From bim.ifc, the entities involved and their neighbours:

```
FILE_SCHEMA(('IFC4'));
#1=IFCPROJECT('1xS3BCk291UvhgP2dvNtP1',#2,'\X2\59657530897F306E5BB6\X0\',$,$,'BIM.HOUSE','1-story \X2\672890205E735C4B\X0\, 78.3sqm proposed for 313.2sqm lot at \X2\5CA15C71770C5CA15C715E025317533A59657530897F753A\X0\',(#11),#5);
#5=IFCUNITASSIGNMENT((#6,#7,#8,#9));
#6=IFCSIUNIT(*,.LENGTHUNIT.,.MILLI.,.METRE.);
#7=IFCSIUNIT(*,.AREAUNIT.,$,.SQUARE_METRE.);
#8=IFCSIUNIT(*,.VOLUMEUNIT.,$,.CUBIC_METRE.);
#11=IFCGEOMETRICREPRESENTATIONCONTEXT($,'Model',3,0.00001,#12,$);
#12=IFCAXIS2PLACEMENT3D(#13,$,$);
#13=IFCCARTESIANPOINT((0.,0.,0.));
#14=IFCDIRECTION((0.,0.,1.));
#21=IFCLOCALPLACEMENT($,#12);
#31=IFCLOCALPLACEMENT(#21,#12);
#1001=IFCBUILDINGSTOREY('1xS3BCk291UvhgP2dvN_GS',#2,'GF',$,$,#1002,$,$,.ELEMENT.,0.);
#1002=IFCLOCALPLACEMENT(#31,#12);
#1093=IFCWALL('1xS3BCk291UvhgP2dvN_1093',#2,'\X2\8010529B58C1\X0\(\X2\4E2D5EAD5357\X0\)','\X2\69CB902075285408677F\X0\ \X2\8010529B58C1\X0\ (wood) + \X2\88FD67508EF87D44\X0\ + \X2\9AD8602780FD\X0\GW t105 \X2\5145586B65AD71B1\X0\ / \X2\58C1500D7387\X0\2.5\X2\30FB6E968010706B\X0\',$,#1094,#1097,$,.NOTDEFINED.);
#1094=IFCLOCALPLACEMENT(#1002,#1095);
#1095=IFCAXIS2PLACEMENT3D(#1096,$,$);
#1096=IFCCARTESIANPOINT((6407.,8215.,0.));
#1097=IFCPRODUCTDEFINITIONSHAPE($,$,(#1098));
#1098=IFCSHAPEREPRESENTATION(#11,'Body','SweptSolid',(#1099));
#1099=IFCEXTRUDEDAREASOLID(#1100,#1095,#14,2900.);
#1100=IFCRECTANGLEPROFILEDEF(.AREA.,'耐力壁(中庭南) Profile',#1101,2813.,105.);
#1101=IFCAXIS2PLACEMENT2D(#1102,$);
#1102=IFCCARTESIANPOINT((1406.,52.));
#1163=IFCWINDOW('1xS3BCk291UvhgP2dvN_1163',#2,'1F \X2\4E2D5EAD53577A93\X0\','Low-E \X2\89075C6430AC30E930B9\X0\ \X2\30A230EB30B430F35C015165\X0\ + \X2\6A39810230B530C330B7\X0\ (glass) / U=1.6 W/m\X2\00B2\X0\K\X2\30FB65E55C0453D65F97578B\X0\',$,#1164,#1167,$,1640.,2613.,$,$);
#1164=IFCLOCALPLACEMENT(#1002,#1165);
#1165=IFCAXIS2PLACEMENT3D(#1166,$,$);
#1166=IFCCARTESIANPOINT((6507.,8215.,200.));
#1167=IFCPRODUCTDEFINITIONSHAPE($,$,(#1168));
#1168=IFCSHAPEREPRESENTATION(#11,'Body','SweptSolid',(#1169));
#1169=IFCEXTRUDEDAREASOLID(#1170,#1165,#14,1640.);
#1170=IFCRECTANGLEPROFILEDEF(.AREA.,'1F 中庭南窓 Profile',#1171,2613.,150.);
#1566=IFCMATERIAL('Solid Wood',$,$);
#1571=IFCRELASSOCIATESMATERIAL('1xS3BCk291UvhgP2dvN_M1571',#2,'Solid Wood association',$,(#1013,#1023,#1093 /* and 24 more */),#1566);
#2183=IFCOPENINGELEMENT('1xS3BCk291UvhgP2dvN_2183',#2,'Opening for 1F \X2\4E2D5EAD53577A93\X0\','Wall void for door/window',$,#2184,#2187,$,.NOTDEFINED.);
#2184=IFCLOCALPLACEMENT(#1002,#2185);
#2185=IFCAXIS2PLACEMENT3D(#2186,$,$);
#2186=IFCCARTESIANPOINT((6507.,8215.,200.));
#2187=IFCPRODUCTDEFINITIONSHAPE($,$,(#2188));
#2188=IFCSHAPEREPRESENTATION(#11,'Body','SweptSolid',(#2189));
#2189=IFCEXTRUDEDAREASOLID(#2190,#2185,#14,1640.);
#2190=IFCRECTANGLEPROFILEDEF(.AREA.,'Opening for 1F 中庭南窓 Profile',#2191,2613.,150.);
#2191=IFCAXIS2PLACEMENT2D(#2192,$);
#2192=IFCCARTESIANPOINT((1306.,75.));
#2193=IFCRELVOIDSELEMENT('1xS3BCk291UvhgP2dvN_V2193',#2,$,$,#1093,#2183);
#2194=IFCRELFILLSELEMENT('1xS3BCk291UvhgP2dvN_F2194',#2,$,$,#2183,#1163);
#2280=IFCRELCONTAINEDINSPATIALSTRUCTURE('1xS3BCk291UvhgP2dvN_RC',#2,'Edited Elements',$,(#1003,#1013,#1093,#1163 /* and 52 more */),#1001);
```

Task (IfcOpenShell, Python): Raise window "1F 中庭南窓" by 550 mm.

```python
import numpy as np
import ifcopenshell
import ifcopenshell.api.geometry
import ifcopenshell.util.placement
import ifcopenshell.util.unit

model = ifcopenshell.open("bim.ifc")
unit_scale = ifcopenshell.util.unit.calculate_unit_scale(model)

window = model.by_guid("1xS3BCk291UvhgP2dvN_1163")
opening = window.FillsVoids[0].RelatingOpeningElement
dz = 550.0

shift = np.array([0.0, 0.0, dz])
# The window is not placed relative to its opening, so move both.
for product in (opening, window):
    matrix = ifcopenshell.util.placement.get_local_placement(product.ObjectPlacement)
    matrix[:3, 3] += shift
    ifcopenshell.api.geometry.edit_object_placement(model, product=product, matrix=matrix, is_si=False)

print(f"moved by {dz * unit_scale:+.3f} m")

model.write("bim_v2.ifc")
```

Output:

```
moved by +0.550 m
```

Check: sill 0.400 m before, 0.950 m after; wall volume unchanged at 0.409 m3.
